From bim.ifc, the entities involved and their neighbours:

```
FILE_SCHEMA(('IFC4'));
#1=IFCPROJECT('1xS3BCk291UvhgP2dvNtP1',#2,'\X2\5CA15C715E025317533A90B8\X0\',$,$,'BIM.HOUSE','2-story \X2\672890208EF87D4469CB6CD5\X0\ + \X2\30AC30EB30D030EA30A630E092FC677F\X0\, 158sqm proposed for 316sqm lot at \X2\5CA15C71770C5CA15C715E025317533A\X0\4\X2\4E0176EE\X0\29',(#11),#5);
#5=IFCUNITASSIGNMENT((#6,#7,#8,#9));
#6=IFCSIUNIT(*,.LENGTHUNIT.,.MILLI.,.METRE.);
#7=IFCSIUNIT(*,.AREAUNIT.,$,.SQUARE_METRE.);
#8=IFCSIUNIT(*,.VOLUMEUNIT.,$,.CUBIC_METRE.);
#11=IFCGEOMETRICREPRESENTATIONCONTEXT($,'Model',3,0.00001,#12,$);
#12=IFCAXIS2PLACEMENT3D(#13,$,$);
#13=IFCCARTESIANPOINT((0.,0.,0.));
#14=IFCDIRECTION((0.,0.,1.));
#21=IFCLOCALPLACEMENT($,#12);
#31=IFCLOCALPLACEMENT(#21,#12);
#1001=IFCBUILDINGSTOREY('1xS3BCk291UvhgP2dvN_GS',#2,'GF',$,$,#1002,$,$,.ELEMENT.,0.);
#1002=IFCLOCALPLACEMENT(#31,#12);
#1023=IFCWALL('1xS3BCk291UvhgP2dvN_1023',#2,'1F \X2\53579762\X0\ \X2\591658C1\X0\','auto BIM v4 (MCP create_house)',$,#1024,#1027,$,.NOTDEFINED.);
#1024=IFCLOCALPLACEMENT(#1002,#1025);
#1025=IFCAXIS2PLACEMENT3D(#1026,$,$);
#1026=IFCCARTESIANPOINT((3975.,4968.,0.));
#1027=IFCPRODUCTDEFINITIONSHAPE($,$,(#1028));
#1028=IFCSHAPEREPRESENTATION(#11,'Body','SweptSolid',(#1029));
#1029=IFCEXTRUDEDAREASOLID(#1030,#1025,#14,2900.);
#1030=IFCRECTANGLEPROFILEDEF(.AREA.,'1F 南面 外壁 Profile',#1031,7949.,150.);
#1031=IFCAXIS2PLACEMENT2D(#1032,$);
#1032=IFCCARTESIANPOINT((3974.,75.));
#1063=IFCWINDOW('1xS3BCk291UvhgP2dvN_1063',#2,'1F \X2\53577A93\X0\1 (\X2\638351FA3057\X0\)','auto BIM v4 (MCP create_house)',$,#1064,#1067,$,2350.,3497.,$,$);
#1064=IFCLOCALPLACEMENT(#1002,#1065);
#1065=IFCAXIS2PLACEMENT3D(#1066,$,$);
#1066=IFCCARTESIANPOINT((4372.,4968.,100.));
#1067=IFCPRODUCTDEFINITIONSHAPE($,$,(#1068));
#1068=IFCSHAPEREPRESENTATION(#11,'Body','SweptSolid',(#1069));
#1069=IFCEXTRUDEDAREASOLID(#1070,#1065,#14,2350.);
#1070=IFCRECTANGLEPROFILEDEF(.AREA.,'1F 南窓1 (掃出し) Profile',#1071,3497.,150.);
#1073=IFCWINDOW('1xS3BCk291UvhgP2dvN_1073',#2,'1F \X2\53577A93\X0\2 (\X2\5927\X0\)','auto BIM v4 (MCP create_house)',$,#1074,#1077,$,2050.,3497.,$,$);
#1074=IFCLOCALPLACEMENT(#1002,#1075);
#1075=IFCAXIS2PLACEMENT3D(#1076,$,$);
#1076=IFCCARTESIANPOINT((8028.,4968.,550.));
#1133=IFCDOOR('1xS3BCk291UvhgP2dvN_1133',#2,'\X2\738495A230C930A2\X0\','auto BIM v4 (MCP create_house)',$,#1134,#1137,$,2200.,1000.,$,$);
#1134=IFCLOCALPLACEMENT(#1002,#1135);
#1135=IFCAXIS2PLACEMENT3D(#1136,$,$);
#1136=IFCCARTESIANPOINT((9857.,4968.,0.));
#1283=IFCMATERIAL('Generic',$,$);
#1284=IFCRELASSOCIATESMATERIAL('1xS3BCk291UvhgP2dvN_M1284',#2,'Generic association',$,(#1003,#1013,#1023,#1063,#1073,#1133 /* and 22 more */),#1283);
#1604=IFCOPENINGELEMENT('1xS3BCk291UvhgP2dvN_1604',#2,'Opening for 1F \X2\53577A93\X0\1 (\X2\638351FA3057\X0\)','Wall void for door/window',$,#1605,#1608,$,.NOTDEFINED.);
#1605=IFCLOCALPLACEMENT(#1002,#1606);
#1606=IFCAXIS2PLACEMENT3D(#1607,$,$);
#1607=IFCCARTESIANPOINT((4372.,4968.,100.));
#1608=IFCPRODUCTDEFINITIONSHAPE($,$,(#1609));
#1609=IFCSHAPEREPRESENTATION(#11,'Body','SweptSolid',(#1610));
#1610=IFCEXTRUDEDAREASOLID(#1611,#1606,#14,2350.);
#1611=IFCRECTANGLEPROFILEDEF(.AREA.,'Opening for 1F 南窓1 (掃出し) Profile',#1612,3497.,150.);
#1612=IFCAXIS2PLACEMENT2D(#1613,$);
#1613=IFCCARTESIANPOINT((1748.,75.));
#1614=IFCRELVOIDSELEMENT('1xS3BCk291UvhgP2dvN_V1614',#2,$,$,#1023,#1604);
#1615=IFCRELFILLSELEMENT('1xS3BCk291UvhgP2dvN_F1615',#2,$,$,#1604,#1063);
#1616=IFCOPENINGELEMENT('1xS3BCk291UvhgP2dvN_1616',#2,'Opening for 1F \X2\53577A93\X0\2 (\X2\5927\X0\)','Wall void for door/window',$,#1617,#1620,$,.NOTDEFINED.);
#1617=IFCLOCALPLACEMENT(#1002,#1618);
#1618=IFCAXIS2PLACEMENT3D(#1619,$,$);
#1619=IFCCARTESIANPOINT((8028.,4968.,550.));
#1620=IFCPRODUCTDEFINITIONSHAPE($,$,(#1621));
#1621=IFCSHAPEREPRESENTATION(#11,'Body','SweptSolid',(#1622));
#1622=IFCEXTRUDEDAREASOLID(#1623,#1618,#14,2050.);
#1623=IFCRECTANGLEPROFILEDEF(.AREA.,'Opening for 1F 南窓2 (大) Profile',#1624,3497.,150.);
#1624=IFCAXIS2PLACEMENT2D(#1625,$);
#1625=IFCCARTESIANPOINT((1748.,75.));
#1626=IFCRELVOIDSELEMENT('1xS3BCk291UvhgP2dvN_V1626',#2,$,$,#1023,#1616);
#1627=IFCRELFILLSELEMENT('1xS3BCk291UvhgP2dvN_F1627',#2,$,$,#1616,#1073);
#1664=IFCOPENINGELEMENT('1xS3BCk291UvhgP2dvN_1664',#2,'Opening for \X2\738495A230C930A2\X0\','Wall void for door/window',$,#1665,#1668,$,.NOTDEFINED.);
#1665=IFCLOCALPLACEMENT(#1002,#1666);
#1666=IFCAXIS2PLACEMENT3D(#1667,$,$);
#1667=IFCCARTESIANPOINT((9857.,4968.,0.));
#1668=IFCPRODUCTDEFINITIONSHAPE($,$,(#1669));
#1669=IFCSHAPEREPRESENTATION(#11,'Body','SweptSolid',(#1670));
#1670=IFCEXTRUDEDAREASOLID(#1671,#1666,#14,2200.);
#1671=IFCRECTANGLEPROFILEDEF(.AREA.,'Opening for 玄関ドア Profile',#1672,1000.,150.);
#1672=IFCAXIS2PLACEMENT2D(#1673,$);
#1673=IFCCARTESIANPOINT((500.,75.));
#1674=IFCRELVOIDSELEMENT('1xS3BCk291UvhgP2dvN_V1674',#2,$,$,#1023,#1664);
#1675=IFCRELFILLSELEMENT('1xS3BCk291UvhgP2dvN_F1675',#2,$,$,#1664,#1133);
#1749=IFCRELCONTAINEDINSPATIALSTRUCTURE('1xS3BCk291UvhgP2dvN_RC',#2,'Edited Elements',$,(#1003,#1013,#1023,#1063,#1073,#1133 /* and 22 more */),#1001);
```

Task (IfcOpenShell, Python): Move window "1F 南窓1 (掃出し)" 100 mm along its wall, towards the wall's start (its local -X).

```python
import ifcopenshell
import ifcopenshell.api.geometry
import ifcopenshell.util.placement
import ifcopenshell.util.unit

model = ifcopenshell.open("bim.ifc")
unit_scale = ifcopenshell.util.unit.calculate_unit_scale(model)

window = model.by_guid("1xS3BCk291UvhgP2dvN_1063")
opening = window.FillsVoids[0].RelatingOpeningElement
wall = opening.VoidsElements[0].RelatingBuildingElement

wall_matrix = ifcopenshell.util.placement.get_local_placement(wall.ObjectPlacement)
shift = wall_matrix[:3, 0] * -0.1 / unit_scale
before = ifcopenshell.util.placement.get_local_placement(window.ObjectPlacement)[:3, 3].copy()

# The window is not placed relative to its opening, so move both.
for product in (opening, window):
    matrix = ifcopenshell.util.placement.get_local_placement(product.ObjectPlacement)
    matrix[:3, 3] += shift
    ifcopenshell.api.geometry.edit_object_placement(model, product=product, matrix=matrix, is_si=False)

after = ifcopenshell.util.placement.get_local_placement(window.ObjectPlacement)[:3, 3]
print("window moved by", (after - before).round(3) + 0.0)

model.write("bim-out.ifc")
```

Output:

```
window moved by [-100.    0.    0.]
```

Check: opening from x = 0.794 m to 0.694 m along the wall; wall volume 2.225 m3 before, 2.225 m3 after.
